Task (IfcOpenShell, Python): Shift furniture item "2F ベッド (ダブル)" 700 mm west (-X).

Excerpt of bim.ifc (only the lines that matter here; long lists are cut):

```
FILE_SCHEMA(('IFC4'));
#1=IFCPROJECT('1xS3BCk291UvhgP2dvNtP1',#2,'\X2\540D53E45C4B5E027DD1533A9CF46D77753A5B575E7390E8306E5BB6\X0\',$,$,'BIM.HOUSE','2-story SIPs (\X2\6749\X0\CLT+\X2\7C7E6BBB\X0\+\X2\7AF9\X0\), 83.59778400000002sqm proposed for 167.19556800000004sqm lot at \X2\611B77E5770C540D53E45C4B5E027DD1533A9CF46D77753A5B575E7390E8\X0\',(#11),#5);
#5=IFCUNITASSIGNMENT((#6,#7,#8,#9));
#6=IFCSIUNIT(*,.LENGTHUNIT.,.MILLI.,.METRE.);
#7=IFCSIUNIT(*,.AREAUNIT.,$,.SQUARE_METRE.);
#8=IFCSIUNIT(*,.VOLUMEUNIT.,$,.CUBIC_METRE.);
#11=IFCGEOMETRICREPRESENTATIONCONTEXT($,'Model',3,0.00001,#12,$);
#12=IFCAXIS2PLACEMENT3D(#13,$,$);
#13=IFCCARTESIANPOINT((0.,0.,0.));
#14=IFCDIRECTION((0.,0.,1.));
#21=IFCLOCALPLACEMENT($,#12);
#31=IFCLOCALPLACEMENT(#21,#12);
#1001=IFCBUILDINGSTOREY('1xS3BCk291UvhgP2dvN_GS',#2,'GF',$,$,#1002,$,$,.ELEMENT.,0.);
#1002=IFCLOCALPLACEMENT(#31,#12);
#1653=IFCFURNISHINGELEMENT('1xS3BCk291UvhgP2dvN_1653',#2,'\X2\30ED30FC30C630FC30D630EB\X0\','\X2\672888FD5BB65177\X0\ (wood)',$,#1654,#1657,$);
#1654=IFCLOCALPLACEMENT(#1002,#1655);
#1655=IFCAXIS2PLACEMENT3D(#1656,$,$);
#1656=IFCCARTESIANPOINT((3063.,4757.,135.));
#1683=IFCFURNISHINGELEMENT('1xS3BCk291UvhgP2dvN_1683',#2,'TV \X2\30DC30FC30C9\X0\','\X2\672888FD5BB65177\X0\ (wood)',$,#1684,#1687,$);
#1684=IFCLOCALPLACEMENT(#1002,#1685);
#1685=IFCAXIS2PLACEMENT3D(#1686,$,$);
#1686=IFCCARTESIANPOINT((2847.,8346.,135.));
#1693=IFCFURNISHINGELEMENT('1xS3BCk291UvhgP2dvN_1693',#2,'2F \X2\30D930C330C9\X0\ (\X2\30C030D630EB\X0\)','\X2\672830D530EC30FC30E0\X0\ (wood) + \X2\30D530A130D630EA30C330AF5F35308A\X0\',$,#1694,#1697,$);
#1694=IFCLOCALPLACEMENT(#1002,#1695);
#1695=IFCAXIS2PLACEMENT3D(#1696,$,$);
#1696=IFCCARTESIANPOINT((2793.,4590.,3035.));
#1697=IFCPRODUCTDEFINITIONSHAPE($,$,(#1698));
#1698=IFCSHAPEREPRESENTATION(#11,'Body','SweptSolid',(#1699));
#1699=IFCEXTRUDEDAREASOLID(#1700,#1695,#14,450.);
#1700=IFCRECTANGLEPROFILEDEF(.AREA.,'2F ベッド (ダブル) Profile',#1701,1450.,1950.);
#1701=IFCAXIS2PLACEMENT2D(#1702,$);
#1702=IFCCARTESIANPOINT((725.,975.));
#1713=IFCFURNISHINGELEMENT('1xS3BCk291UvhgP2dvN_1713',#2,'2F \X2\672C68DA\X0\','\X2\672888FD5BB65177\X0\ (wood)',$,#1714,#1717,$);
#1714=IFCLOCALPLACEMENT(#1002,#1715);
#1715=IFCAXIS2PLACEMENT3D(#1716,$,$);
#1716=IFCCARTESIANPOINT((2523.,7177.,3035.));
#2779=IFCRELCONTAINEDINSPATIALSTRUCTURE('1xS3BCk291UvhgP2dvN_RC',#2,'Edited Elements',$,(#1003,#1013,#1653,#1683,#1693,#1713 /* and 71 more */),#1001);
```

```python
import ifcopenshell
import ifcopenshell.api.geometry
import ifcopenshell.util.placement
import ifcopenshell.util.unit

model = ifcopenshell.open("bim.ifc")
unit_scale = ifcopenshell.util.unit.calculate_unit_scale(model)

item = model.by_guid("1xS3BCk291UvhgP2dvN_1693")
matrix = ifcopenshell.util.placement.get_local_placement(item.ObjectPlacement)
matrix[0, 3] -= 0.7 / unit_scale
ifcopenshell.api.geometry.edit_object_placement(model, product=item, matrix=matrix, is_si=False)

print(ifcopenshell.util.placement.get_local_placement(item.ObjectPlacement).round(3) + 0.0)

model.write("bim_v2.ifc")
```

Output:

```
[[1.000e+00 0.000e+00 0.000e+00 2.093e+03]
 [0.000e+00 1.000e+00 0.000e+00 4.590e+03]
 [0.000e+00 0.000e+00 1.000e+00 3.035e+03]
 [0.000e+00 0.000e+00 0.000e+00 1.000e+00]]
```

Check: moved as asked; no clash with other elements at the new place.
